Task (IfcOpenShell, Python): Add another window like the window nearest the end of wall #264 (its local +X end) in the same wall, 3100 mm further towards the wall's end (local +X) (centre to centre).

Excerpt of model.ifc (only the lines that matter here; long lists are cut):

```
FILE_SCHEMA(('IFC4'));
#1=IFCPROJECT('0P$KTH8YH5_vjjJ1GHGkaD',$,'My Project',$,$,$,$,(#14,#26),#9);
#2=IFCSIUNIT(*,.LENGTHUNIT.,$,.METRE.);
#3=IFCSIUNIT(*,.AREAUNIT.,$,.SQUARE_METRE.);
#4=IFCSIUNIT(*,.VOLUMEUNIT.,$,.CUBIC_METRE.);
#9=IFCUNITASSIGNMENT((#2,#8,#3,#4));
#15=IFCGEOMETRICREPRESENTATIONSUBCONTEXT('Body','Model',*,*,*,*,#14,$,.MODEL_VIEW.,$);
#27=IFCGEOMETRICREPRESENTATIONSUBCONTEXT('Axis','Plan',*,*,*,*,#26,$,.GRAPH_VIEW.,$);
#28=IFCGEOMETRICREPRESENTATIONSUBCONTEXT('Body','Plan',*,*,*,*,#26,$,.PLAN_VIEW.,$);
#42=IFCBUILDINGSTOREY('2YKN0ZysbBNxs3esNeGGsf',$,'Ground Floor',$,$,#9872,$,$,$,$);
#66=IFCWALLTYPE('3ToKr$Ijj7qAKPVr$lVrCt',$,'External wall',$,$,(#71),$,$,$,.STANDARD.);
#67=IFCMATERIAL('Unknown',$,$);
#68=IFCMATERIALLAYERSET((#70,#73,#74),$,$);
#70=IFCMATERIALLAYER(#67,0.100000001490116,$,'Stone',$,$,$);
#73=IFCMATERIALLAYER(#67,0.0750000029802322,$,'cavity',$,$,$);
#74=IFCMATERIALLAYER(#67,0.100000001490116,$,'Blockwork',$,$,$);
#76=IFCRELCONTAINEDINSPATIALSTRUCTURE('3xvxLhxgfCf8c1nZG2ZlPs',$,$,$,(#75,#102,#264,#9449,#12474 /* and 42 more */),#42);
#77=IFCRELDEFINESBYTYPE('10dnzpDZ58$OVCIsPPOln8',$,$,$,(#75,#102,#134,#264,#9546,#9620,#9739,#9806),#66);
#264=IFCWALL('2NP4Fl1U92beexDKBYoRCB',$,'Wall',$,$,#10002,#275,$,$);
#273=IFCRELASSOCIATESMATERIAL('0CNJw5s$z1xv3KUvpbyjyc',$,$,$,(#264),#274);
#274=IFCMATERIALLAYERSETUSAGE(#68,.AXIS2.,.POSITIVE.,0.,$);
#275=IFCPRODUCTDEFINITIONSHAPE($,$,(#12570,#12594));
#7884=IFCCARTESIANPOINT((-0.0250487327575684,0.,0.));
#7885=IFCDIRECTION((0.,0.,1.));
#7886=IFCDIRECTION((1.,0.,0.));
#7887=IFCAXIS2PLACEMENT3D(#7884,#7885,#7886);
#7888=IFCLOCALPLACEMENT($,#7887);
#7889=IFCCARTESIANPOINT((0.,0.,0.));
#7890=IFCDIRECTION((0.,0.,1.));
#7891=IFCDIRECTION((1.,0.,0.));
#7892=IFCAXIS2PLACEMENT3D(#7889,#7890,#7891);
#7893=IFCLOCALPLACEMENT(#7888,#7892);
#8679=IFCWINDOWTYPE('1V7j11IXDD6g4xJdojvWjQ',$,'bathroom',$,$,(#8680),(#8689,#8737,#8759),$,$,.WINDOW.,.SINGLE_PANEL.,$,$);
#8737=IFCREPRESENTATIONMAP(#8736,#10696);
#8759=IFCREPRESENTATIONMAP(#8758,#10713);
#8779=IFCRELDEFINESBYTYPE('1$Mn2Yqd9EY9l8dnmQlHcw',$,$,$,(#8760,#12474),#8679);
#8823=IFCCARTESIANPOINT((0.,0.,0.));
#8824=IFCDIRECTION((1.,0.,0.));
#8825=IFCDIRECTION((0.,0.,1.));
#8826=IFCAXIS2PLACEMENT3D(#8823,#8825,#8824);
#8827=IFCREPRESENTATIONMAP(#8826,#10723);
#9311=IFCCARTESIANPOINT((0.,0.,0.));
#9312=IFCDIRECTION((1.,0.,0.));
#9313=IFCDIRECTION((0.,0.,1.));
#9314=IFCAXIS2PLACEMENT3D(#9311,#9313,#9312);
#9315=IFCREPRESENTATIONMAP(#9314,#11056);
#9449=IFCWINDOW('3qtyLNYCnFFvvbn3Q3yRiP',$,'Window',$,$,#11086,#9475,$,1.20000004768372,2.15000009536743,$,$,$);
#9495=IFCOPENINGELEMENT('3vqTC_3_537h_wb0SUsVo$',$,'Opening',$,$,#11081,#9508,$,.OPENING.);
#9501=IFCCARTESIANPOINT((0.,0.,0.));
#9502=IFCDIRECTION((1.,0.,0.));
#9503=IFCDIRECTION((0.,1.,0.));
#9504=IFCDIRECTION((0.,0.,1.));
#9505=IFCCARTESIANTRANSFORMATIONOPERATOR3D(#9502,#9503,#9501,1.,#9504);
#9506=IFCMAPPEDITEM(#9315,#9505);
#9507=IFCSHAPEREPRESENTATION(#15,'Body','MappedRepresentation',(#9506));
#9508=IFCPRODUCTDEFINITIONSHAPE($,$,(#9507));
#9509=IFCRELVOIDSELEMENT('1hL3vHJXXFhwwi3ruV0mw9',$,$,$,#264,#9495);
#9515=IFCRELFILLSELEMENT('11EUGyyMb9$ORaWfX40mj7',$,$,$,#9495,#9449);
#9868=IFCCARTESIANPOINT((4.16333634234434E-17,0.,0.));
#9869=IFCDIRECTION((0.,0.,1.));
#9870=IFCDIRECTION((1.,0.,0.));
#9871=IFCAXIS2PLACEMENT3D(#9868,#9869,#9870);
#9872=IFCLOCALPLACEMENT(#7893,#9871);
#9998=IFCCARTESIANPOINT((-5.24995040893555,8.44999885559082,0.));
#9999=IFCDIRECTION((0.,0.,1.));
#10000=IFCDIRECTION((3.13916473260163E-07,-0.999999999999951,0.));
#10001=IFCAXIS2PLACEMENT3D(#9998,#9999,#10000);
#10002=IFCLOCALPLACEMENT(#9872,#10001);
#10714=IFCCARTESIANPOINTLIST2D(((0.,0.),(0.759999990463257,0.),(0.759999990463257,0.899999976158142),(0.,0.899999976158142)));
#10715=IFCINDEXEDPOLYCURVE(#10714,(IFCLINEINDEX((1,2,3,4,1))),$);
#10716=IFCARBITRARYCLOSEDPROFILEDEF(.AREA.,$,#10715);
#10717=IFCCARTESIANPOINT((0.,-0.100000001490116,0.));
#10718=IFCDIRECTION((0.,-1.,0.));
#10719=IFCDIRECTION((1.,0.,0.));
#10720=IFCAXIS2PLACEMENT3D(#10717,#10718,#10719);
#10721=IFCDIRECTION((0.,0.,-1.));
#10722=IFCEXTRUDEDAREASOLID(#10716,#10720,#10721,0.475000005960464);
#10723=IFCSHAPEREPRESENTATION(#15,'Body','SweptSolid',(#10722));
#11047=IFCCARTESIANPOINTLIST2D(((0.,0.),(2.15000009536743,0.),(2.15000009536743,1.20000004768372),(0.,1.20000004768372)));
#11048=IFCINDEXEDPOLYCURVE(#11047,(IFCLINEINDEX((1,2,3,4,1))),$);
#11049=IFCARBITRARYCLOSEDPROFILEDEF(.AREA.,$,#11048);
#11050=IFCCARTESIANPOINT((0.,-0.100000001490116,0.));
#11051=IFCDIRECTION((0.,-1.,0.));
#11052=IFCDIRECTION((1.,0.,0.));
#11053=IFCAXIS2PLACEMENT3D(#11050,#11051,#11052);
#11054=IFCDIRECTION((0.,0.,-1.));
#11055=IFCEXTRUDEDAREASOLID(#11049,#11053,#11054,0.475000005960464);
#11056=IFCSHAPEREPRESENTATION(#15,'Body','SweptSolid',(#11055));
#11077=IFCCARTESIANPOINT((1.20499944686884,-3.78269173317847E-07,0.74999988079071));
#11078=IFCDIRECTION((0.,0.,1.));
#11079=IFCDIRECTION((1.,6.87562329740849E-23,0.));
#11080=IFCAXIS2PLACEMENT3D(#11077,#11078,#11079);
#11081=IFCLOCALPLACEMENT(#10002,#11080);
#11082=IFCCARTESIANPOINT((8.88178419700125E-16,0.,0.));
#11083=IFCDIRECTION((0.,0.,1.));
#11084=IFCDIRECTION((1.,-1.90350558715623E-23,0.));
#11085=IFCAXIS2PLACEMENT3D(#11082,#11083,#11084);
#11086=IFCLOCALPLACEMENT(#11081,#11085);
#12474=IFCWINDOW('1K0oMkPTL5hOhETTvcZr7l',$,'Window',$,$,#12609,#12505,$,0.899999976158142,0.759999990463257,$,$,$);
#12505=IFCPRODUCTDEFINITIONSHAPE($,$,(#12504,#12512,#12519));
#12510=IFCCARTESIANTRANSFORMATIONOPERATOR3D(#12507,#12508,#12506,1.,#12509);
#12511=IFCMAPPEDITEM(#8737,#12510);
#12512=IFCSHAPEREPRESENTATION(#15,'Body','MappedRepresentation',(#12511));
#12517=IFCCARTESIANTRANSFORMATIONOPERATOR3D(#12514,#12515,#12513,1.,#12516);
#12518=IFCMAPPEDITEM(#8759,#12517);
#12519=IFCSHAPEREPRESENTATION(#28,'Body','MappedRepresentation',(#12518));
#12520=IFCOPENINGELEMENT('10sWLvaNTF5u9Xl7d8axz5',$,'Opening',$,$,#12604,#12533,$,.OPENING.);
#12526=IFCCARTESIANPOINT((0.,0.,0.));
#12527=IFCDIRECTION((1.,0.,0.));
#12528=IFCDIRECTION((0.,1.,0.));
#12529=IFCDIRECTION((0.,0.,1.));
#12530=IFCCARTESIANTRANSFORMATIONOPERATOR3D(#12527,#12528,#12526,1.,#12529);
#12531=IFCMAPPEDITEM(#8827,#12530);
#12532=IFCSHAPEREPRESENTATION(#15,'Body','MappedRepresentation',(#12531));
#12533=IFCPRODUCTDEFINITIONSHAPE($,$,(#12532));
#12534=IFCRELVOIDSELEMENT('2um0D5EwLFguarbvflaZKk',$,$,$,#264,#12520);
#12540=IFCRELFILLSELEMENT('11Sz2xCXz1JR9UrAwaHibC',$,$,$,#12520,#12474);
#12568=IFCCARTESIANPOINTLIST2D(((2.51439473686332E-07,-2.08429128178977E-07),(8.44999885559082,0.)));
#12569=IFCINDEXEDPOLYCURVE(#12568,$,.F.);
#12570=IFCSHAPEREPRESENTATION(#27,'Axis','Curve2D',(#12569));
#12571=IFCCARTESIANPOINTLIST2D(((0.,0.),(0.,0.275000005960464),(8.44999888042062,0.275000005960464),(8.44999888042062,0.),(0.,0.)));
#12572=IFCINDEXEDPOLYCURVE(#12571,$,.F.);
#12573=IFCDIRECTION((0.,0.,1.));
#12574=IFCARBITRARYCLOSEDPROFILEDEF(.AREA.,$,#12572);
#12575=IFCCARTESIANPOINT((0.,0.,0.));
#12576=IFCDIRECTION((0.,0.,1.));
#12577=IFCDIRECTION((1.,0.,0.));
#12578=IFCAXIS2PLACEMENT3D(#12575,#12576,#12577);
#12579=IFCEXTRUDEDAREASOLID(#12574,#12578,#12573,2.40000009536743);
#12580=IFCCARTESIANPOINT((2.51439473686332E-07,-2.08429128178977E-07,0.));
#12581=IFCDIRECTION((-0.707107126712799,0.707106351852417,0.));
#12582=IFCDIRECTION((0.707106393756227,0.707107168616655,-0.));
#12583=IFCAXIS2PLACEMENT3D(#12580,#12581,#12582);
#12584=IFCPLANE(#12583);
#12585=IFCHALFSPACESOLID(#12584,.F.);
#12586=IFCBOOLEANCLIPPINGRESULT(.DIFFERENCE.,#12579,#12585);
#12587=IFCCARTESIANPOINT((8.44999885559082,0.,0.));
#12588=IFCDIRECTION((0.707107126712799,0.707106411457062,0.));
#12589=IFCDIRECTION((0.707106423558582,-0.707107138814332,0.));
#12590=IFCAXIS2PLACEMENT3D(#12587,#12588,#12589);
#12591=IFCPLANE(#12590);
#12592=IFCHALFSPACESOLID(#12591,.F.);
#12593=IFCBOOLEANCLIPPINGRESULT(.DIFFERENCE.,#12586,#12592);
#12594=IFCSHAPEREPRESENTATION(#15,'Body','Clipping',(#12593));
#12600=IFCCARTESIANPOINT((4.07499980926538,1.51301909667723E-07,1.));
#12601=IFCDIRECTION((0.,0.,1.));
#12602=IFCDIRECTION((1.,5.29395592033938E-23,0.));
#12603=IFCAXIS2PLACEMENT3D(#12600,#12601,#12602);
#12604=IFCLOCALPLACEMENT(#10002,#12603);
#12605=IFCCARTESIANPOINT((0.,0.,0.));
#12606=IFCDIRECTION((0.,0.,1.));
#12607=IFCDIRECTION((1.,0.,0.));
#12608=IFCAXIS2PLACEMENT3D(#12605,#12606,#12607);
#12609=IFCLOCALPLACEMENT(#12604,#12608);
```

```python
import ifcopenshell
import ifcopenshell.api.feature
import ifcopenshell.api.geometry
import ifcopenshell.api.root
import ifcopenshell.geom
import ifcopenshell.util.element
import ifcopenshell.util.placement
import ifcopenshell.util.shape

model = ifcopenshell.open("model.ifc")
settings = ifcopenshell.geom.settings()


def volume(element):
    """Net volume in cubic metres, openings subtracted."""
    shape = ifcopenshell.geom.create_shape(settings, element)
    return ifcopenshell.util.shape.get_volume(shape.geometry)


window = model.by_guid("1K0oMkPTL5hOhETTvcZr7l")
opening = window.FillsVoids[0].RelatingOpeningElement
wall = opening.VoidsElements[0].RelatingBuildingElement
before = volume(wall)
shift = ifcopenshell.util.placement.get_local_placement(wall.ObjectPlacement)[:3, 0] * 3.1

# copy_class copies the void relationship, type, container and properties, but no geometry.
new_opening = ifcopenshell.api.root.copy_class(model, product=opening)
new_opening.Representation = ifcopenshell.util.element.copy_deep(
    model, opening.Representation, exclude=["IfcGeometricRepresentationContext", "IfcRepresentationMap"]
)
new_window = ifcopenshell.api.root.copy_class(model, product=window)
new_window.Representation = ifcopenshell.util.element.copy_deep(
    model, window.Representation, exclude=["IfcGeometricRepresentationContext", "IfcRepresentationMap"]
)
ifcopenshell.api.feature.add_filling(model, opening=new_opening, element=new_window)

for old, new in ((opening, new_opening), (window, new_window)):
    matrix = ifcopenshell.util.placement.get_local_placement(old.ObjectPlacement)
    matrix[:3, 3] += shift
    ifcopenshell.api.geometry.edit_object_placement(model, product=new, matrix=matrix, is_si=False)

after = volume(wall)

print(f"wall volume {before:.3f} -> {after:.3f} m3")

model.write("model_edited.ifc")
```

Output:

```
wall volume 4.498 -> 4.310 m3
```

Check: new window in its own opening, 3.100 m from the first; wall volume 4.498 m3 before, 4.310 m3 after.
